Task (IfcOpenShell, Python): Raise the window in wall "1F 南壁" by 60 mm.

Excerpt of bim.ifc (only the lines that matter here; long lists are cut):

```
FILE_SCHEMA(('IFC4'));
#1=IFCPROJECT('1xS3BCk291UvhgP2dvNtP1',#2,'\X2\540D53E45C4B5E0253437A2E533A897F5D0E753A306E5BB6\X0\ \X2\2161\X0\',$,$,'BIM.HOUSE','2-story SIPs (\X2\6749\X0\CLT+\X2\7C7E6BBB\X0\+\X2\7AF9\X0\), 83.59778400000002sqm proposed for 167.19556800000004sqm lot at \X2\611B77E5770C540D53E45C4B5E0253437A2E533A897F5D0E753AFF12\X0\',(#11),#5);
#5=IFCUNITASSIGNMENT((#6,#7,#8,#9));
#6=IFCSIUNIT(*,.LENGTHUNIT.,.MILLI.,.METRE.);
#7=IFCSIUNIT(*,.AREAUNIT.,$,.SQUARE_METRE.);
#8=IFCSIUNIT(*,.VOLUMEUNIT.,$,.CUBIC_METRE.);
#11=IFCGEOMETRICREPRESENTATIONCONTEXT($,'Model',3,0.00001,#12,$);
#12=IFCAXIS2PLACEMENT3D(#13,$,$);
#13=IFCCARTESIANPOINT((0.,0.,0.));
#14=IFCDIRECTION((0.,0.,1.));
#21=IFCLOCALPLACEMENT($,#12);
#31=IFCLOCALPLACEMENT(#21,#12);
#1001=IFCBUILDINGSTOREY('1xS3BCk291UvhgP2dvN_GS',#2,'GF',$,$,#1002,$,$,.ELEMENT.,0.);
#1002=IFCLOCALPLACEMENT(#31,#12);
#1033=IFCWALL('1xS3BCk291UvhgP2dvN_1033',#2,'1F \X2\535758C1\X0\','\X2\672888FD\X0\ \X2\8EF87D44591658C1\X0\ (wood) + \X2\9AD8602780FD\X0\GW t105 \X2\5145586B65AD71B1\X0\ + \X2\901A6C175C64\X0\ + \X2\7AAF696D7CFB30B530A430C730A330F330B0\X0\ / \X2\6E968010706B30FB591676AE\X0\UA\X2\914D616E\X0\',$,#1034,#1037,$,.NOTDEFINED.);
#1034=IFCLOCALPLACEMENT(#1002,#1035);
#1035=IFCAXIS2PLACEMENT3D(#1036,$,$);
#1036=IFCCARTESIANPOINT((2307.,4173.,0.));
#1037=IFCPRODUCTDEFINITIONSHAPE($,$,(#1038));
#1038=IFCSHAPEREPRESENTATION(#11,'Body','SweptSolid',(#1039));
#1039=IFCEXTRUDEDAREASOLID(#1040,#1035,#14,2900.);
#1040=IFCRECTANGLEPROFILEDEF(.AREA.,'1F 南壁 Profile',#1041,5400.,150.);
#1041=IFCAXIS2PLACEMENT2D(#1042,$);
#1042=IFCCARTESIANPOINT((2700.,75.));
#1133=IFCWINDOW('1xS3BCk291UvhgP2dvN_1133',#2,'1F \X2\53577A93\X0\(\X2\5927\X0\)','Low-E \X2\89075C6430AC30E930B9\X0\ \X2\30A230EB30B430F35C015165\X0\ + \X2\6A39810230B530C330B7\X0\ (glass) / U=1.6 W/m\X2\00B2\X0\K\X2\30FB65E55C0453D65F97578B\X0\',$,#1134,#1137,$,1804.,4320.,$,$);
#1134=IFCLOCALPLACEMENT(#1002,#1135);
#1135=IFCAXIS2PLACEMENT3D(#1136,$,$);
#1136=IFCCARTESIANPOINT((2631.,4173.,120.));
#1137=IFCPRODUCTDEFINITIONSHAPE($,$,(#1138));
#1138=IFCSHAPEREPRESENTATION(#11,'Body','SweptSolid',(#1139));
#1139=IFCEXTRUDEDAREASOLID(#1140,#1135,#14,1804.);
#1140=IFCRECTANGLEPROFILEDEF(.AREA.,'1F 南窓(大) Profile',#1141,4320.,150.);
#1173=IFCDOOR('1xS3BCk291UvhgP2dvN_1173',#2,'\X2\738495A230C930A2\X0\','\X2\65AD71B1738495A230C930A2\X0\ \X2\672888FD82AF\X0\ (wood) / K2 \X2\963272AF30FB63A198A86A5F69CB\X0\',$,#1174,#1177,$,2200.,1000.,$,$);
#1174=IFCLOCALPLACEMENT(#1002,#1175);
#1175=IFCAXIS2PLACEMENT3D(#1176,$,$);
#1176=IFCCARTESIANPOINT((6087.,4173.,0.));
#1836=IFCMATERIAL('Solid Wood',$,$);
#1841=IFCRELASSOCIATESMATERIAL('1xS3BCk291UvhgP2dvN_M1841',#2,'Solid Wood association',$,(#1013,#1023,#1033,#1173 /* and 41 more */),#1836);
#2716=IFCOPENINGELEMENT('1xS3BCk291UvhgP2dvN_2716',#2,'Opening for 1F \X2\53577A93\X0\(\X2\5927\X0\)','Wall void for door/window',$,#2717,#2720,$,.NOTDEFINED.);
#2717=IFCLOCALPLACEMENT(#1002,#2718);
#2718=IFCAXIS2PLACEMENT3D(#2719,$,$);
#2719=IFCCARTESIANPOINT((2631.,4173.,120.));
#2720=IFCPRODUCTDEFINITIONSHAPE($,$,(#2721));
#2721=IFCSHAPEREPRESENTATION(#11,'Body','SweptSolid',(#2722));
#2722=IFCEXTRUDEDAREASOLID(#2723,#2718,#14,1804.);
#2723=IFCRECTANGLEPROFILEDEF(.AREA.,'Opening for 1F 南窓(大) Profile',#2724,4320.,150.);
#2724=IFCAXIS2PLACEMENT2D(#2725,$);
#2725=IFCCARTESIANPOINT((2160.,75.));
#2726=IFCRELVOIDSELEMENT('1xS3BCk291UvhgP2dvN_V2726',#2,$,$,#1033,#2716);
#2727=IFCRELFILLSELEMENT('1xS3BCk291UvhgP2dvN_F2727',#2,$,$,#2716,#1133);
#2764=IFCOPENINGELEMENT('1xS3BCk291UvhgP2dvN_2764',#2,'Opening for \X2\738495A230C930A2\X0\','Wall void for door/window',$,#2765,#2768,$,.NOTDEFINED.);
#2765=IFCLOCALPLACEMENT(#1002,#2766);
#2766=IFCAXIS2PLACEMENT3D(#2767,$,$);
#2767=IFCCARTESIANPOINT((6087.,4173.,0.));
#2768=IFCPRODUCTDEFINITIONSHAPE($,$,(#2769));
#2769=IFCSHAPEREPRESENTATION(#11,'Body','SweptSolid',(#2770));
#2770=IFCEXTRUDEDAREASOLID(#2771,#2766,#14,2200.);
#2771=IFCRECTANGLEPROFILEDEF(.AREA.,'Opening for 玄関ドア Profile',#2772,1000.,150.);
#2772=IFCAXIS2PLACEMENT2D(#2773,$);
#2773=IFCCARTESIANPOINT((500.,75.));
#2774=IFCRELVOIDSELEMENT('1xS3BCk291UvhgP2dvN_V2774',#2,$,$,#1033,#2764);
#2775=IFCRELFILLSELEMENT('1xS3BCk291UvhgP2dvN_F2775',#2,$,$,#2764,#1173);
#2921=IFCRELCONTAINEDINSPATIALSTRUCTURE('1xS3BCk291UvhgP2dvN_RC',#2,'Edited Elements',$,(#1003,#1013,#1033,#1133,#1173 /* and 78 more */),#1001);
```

```python
import numpy as np
import ifcopenshell
import ifcopenshell.api.geometry
import ifcopenshell.util.placement
import ifcopenshell.util.unit

model = ifcopenshell.open("bim.ifc")
unit_scale = ifcopenshell.util.unit.calculate_unit_scale(model)

window = model.by_id(1133)
opening = window.FillsVoids[0].RelatingOpeningElement
dz = 0.06 / unit_scale

shift = np.array([0.0, 0.0, dz])
# The window is not placed relative to its opening, so move both.
for product in (opening, window):
    matrix = ifcopenshell.util.placement.get_local_placement(product.ObjectPlacement)
    matrix[:3, 3] += shift
    ifcopenshell.api.geometry.edit_object_placement(model, product=product, matrix=matrix, is_si=False)

print(f"moved by {dz * unit_scale:+.3f} m")

model.write("bim_edited.ifc")
```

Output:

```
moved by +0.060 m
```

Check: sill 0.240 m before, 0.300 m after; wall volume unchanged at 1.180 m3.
